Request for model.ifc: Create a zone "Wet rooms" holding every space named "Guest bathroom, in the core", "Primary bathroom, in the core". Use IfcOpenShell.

First a look at what the model holds.

```python
import ifcopenshell

model = ifcopenshell.open("model.ifc")
print(model.schema)
seen = {}
for space in model.by_type("IfcSpace"):
    seen[space.LongName] = seen.get(space.LongName, 0) + 1
for name, count in sorted(seen.items(), key=str):
    print(count, "x", name)
print("zones:", [z.Name for z in model.by_type("IfcZone")][:20])
```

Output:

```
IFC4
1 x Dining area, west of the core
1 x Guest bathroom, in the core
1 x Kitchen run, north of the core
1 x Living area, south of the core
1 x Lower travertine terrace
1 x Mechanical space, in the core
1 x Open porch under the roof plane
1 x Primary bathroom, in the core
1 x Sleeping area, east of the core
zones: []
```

```python
import ifcopenshell
import ifcopenshell.api.group
import ifcopenshell.api.root

model = ifcopenshell.open("model.ifc")

names = {"Guest bathroom, in the core", "Primary bathroom, in the core"}
spaces = [s for s in model.by_type("IfcSpace") if s.LongName in names]

zone = ifcopenshell.api.root.create_entity(model, ifc_class="IfcZone", name="Wet rooms")
ifcopenshell.api.group.assign_group(model, products=spaces, group=zone)
print(len(spaces), "spaces in", zone.Name)

model.write("model-out.ifc")
```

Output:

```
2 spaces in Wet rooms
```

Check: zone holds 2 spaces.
